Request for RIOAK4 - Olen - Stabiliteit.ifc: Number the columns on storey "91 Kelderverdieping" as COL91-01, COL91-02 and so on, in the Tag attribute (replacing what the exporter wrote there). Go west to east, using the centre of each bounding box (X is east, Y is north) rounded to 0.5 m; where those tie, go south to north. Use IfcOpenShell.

First a look at what the model holds.

```python
import ifcopenshell
import ifcopenshell.util.element
import ifcopenshell.util.placement

model = ifcopenshell.open("RIOAK4 - Olen - Stabiliteit.ifc")
print(model.schema)
storey = next(s for s in model.by_type("IfcBuildingStorey") if s.Name == "91 Kelderverdieping")
columns = [e for e in ifcopenshell.util.element.get_decomposition(storey) if e.is_a("IfcColumn")]
for e in sorted(columns, key=lambda e: e.id()):
    origin = ifcopenshell.util.placement.get_local_placement(e.ObjectPlacement)[:3, 3]
    print(e.id(), e.Tag, e.Name, origin.round(2) + 0.0, sep=" | ")
```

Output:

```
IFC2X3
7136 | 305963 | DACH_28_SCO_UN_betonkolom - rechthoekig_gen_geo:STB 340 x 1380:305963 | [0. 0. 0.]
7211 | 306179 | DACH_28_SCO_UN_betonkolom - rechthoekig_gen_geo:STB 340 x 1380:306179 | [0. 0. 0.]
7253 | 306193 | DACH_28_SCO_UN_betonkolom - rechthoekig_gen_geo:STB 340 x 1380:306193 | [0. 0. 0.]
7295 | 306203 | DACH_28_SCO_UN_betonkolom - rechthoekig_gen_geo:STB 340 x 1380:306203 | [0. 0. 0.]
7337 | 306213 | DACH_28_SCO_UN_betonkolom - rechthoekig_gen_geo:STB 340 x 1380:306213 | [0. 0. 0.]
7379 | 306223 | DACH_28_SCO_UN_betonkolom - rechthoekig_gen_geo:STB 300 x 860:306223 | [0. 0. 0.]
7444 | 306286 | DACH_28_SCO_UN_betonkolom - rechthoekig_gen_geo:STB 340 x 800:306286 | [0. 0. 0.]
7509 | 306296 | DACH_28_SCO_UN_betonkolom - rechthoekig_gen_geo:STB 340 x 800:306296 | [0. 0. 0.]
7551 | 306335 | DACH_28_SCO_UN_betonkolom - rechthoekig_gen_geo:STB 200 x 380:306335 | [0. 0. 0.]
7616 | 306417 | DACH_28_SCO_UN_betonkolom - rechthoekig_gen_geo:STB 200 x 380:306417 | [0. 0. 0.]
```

```python
import ifcopenshell
import ifcopenshell.geom
import ifcopenshell.util.element
import ifcopenshell.util.shape

model = ifcopenshell.open("RIOAK4 - Olen - Stabiliteit.ifc")
settings = ifcopenshell.geom.settings()
settings.set("use-world-coords", True)


def centre(element):
    shape = ifcopenshell.geom.create_shape(settings, element)
    return ifcopenshell.util.shape.get_bbox_centroid(shape.geometry)


storey = next(s for s in model.by_type("IfcBuildingStorey") if s.Name == "91 Kelderverdieping")
columns = [e for e in ifcopenshell.util.element.get_decomposition(storey) if e.is_a("IfcColumn")]

# Insertion points can sit at a corner or the storey origin, so sort by the geometry (in metres).
centres = {e: centre(e) for e in columns}
columns.sort(key=lambda e: (round(centres[e][0] / 0.5), centres[e][1]))

for i, e in enumerate(columns, start=1):
    number = f"COL91-{i:02d}"
    e.Tag = number
    print(e.id(), number)

model.write("RIOAK4 - Olen - Stabiliteit_edited.ifc")
```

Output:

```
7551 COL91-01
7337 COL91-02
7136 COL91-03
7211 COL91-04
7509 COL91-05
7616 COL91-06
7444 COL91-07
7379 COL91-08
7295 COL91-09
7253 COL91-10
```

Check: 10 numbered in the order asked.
